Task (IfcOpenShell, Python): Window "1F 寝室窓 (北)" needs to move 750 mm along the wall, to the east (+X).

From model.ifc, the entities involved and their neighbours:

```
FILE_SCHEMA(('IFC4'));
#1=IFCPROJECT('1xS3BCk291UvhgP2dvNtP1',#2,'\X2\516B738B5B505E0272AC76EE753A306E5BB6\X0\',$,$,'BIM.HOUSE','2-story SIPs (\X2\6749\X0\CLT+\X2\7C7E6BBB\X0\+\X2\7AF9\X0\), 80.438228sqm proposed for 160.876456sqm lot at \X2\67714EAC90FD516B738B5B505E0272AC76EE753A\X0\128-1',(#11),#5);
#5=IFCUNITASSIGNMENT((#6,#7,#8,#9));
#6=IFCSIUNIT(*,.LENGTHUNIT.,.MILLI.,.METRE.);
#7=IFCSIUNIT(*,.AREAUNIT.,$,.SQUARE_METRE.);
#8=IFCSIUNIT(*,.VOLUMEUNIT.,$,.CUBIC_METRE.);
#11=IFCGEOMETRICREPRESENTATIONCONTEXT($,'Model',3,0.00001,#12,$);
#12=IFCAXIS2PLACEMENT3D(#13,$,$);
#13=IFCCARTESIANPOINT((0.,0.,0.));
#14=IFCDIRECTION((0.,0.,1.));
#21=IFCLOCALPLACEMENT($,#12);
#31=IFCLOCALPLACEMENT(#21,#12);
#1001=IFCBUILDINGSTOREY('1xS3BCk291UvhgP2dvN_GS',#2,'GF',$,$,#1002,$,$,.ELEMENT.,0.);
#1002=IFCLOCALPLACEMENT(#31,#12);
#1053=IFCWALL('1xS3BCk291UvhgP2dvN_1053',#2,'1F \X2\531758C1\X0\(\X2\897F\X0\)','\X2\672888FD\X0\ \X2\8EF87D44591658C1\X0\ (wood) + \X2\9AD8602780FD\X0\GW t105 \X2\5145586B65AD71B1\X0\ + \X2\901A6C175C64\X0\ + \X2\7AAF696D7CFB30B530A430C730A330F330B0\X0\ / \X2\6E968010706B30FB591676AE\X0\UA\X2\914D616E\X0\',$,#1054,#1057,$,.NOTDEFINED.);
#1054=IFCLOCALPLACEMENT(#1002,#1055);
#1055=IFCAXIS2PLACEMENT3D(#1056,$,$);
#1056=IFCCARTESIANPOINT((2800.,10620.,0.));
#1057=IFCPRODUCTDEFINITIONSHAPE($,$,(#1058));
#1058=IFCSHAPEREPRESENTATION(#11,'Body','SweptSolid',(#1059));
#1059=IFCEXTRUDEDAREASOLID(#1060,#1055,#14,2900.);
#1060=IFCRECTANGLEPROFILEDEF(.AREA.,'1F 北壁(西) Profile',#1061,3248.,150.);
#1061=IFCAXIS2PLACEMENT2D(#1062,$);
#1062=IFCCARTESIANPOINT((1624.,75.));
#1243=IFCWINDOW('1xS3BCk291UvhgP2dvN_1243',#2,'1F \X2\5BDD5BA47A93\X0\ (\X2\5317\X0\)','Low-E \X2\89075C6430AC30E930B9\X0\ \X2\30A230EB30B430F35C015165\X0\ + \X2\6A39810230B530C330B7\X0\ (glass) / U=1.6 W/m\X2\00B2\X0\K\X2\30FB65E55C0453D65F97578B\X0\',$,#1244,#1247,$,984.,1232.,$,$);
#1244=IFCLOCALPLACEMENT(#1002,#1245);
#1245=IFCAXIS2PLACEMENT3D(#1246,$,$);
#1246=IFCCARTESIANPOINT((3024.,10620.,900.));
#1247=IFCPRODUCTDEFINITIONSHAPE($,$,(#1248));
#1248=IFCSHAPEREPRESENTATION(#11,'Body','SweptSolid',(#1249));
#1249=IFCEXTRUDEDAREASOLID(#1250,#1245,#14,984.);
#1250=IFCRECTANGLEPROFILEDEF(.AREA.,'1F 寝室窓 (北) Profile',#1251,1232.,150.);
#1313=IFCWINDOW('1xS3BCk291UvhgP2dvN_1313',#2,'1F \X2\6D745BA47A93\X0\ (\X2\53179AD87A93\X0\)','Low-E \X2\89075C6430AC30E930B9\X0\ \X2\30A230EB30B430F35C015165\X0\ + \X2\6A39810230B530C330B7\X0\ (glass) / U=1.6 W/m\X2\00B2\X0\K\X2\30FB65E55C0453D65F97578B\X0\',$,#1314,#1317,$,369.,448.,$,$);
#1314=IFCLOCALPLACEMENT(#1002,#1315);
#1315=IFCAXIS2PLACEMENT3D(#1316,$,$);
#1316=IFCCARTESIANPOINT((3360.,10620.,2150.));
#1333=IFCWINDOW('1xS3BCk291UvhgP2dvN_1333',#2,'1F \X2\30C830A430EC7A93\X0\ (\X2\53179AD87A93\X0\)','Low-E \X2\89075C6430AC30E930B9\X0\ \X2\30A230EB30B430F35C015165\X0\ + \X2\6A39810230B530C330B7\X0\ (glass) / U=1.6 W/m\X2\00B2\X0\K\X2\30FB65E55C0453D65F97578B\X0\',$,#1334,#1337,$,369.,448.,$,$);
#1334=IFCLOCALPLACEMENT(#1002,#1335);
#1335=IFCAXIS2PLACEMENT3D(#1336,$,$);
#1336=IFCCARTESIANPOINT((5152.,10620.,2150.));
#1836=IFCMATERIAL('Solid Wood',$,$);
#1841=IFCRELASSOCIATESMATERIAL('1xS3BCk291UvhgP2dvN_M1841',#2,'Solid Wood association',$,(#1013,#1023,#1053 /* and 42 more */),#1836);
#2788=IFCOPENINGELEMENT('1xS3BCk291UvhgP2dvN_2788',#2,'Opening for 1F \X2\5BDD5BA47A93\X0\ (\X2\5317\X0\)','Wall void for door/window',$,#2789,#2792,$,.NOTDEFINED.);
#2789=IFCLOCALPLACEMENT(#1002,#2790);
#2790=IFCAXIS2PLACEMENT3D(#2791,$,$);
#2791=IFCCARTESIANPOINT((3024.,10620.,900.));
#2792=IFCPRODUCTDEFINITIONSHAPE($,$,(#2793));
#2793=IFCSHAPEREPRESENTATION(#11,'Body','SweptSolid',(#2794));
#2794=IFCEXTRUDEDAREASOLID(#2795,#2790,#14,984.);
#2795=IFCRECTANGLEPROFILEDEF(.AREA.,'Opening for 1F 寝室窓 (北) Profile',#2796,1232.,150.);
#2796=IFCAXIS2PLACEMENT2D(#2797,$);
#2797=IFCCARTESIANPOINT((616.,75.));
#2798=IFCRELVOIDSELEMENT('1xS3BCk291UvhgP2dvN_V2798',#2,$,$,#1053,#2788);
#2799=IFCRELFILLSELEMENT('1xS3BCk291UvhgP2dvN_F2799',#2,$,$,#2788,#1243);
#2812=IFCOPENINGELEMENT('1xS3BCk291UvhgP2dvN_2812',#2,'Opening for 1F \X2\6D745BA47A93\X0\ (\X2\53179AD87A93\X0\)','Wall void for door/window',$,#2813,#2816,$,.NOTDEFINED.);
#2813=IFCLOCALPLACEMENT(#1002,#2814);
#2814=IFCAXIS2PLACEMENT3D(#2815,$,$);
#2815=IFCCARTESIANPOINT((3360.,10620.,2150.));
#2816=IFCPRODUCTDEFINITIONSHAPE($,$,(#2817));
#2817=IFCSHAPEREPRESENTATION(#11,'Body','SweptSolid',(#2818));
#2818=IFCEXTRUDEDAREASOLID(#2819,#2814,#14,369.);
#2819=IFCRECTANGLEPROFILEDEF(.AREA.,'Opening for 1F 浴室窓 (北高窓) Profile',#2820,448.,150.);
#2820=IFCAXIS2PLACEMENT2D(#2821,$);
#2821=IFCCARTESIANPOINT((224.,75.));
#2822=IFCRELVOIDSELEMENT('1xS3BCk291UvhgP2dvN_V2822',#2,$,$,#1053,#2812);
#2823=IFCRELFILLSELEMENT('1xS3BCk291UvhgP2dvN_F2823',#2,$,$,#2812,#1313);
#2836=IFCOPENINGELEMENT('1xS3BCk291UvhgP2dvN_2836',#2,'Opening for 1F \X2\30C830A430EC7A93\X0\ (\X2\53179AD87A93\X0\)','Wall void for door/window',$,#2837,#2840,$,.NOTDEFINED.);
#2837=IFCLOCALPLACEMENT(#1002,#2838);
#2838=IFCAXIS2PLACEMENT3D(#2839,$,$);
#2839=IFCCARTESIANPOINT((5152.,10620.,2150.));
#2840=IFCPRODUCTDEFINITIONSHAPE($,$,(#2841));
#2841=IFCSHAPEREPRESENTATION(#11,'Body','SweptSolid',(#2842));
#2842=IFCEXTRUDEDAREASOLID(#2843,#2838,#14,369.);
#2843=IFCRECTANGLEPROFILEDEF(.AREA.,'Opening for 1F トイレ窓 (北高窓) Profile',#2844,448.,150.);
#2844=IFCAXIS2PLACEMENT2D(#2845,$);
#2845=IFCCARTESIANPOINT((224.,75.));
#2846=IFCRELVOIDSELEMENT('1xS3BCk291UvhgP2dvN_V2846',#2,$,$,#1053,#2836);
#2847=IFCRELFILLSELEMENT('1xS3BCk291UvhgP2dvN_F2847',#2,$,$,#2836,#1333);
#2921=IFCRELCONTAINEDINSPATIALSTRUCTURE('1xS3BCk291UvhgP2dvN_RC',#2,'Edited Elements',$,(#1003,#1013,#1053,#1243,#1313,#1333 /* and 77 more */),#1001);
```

```python
import ifcopenshell
import ifcopenshell.api.geometry
import ifcopenshell.util.placement
import ifcopenshell.util.unit

model = ifcopenshell.open("model.ifc")
unit_scale = ifcopenshell.util.unit.calculate_unit_scale(model)

window = model.by_guid("1xS3BCk291UvhgP2dvN_1243")
opening = window.FillsVoids[0].RelatingOpeningElement
wall = opening.VoidsElements[0].RelatingBuildingElement

wall_matrix = ifcopenshell.util.placement.get_local_placement(wall.ObjectPlacement)
shift = wall_matrix[:3, 0] * 0.75 / unit_scale
before = ifcopenshell.util.placement.get_local_placement(window.ObjectPlacement)[:3, 3].copy()

# The window is not placed relative to its opening, so move both.
for product in (opening, window):
    matrix = ifcopenshell.util.placement.get_local_placement(product.ObjectPlacement)
    matrix[:3, 3] += shift
    ifcopenshell.api.geometry.edit_object_placement(model, product=product, matrix=matrix, is_si=False)

after = ifcopenshell.util.placement.get_local_placement(window.ObjectPlacement)[:3, 3]
print("window moved by", (after - before).round(3) + 0.0)

model.write("model-out.ifc")
```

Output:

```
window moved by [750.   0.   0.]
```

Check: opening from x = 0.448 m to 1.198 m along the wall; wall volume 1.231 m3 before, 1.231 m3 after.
